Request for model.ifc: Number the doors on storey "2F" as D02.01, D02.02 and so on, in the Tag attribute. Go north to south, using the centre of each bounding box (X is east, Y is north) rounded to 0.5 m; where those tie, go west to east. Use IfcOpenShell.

First a look at what the model holds.

```python
import ifcopenshell
import ifcopenshell.util.element
import ifcopenshell.util.placement

model = ifcopenshell.open("model.ifc")
print(model.schema)
storey = next(s for s in model.by_type("IfcBuildingStorey") if s.Name == "2F")
doors = [e for e in ifcopenshell.util.element.get_decomposition(storey) if e.is_a("IfcDoor")]
for e in sorted(doors, key=lambda e: e.id()):
    origin = ifcopenshell.util.placement.get_local_placement(e.ObjectPlacement)[:3, 3]
    print(e.id(), e.Tag, e.Name, origin.round(2) + 0.0, sep=" | ")
```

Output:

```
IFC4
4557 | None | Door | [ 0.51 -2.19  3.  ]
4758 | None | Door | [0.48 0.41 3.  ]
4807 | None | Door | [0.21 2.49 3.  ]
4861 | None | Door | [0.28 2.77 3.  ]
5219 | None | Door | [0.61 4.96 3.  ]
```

```python
import ifcopenshell
import ifcopenshell.geom
import ifcopenshell.util.element
import ifcopenshell.util.shape

model = ifcopenshell.open("model.ifc")
settings = ifcopenshell.geom.settings()
settings.set("use-world-coords", True)


def centre(element):
    shape = ifcopenshell.geom.create_shape(settings, element)
    return ifcopenshell.util.shape.get_bbox_centroid(shape.geometry)


storey = next(s for s in model.by_type("IfcBuildingStorey") if s.Name == "2F")
doors = [e for e in ifcopenshell.util.element.get_decomposition(storey) if e.is_a("IfcDoor")]

# Insertion points can sit at a corner or the storey origin, so sort by the geometry (in metres).
centres = {e: centre(e) for e in doors}
doors.sort(key=lambda e: (-round(centres[e][1] / 0.5), centres[e][0]))

for i, e in enumerate(doors, start=1):
    number = f"D02.{i:02d}"
    e.Tag = number
    print(e.id(), number)

model.write("model-out.ifc")
```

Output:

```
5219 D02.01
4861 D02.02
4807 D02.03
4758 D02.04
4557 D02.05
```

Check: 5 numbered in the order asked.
